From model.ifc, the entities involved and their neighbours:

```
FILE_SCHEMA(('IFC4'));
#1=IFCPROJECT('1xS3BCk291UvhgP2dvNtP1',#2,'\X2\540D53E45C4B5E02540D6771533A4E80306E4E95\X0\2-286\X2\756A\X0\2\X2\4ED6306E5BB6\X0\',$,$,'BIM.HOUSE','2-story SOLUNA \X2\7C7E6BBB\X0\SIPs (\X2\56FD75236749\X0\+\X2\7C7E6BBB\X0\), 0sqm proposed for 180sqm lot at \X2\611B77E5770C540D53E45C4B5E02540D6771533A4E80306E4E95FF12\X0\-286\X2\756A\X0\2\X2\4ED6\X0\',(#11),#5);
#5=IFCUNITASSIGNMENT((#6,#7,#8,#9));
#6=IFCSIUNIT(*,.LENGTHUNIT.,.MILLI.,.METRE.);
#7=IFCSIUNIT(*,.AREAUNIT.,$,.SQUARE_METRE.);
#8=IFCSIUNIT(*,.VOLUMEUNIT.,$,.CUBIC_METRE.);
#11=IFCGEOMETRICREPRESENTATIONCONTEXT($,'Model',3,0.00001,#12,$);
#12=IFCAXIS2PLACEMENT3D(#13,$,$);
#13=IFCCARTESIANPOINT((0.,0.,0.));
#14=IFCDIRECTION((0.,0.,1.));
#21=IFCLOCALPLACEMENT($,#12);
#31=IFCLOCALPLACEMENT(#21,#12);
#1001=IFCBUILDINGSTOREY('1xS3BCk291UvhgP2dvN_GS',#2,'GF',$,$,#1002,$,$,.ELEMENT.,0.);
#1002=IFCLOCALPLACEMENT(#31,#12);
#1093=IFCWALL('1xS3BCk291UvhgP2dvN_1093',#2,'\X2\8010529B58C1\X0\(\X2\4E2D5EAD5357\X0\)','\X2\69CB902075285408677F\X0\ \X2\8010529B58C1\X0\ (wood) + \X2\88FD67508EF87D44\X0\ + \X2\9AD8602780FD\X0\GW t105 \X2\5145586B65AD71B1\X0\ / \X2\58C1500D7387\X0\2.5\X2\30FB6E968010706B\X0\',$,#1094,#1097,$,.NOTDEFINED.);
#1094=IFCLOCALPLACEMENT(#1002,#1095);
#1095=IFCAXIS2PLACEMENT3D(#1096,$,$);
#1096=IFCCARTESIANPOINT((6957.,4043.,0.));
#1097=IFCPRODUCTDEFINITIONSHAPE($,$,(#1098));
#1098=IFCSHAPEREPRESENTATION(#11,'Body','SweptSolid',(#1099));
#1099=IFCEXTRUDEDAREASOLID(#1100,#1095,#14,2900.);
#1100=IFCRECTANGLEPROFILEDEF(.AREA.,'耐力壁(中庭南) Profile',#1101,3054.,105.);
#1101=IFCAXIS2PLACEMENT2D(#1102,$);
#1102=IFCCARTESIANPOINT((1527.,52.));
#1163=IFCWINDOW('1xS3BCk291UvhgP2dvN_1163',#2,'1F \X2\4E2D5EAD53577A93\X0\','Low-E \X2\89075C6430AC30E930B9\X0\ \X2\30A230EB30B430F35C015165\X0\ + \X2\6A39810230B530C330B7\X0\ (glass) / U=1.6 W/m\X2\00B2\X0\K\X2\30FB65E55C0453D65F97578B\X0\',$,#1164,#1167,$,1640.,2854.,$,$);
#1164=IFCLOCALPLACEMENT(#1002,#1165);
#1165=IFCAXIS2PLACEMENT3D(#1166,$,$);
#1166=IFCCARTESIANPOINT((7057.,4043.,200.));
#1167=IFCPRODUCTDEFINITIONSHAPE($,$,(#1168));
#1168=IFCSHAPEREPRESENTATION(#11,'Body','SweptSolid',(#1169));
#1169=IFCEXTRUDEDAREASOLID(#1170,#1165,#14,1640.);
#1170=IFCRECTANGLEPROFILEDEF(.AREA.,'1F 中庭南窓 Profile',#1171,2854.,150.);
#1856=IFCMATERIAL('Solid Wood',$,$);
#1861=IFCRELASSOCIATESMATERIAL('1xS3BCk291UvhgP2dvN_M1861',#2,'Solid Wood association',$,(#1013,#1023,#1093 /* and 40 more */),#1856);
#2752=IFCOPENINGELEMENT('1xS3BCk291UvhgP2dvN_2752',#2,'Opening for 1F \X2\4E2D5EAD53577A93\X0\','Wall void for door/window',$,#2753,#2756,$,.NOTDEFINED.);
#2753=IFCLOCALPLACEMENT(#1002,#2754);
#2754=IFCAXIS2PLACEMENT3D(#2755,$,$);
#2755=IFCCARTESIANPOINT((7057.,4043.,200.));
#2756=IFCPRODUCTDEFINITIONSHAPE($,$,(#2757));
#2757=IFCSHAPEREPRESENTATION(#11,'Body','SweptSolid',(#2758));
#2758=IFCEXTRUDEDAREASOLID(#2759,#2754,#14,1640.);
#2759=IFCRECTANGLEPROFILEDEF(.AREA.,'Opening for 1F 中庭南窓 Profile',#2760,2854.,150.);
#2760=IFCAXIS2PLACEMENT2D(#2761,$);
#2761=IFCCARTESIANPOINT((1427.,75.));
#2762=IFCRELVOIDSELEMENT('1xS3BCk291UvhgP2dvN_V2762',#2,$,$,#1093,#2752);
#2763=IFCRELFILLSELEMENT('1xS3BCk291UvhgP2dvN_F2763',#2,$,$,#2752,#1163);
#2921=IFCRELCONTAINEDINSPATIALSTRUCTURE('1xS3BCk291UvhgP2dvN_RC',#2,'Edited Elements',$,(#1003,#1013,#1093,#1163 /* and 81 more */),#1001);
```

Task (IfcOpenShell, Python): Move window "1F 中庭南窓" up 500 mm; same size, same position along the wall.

```python
import numpy as np
import ifcopenshell
import ifcopenshell.api.geometry
import ifcopenshell.util.placement
import ifcopenshell.util.unit

model = ifcopenshell.open("model.ifc")
unit_scale = ifcopenshell.util.unit.calculate_unit_scale(model)

window = model.by_guid("1xS3BCk291UvhgP2dvN_1163")
opening = window.FillsVoids[0].RelatingOpeningElement
dz = 0.5 / unit_scale

shift = np.array([0.0, 0.0, dz])
# The window is not placed relative to its opening, so move both.
for product in (opening, window):
    matrix = ifcopenshell.util.placement.get_local_placement(product.ObjectPlacement)
    matrix[:3, 3] += shift
    ifcopenshell.api.geometry.edit_object_placement(model, product=product, matrix=matrix, is_si=False)

print(f"moved by {dz * unit_scale:+.3f} m")

model.write("model_updated.ifc")
```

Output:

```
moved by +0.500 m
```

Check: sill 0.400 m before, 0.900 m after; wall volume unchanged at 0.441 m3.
